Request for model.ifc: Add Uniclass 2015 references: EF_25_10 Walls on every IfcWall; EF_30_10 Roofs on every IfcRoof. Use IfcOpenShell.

First a look at what the model holds.

```python
import ifcopenshell

model = ifcopenshell.open("model.ifc")
print(model.schema)
print("classifications:", [c.Name for c in model.by_type("IfcClassification")])
for ifc_class in ("IfcDoor", "IfcRoof", "IfcStair", "IfcWall", "IfcWindow"):
    print(ifc_class, len(model.by_type(ifc_class)))
```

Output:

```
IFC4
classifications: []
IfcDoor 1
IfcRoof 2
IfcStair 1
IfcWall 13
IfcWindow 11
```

```python
import ifcopenshell
import ifcopenshell.api.classification

model = ifcopenshell.open("model.ifc")

system = ifcopenshell.api.classification.add_classification(model, classification="Uniclass 2015")

codes = {
    "IfcWall": ("EF_25_10", "Walls"),
    "IfcRoof": ("EF_30_10", "Roofs"),
}
for ifc_class, (code, name) in codes.items():
    products = model.by_type(ifc_class)
    ifcopenshell.api.classification.add_reference(
        model, products=products, classification=system, identification=code, name=name
    )
    print(code, len(products))

model.write("model_rev.ifc")
```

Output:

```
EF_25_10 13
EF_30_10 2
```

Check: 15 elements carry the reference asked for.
